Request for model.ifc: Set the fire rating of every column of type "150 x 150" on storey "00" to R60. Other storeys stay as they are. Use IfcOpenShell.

First a look at what the model holds.

```python
import ifcopenshell
import ifcopenshell.util.element

model = ifcopenshell.open("model.ifc")
print(model.schema)
storey = next(s for s in model.by_type("IfcBuildingStorey") if s.Name == "00")
columns = [e for e in ifcopenshell.util.element.get_decomposition(storey) if e.is_a("IfcColumn")]
seen = {}
for e in columns:
    element_type = ifcopenshell.util.element.get_type(e)
    key = (element_type.Name if element_type != e and element_type else None, ifcopenshell.util.element.get_pset(e, "Pset_ColumnCommon", "FireRating"))
    seen[key] = seen.get(key, 0) + 1
for (name, value), count in sorted(seen.items(), key=str):
    print(count, "x", name, "|", value)
```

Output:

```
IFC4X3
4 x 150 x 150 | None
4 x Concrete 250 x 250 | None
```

```python
import ifcopenshell
import ifcopenshell.api.pset
import ifcopenshell.util.element

model = ifcopenshell.open("model.ifc")

storey = next(s for s in model.by_type("IfcBuildingStorey") if s.Name == "00")
columns = [e for e in ifcopenshell.util.element.get_decomposition(storey) if e.is_a("IfcColumn")]

count = 0
for e in columns:
    element_type = ifcopenshell.util.element.get_type(e)
    if element_type in (None, e) or element_type.Name != "150 x 150":
        continue
    # add_pset returns the element's existing set when there is one.
    pset = ifcopenshell.api.pset.add_pset(model, product=e, name="Pset_ColumnCommon")
    ifcopenshell.api.pset.edit_pset(model, pset=pset, properties={"FireRating": "R60"})
    count += 1

print(count, "columns updated")

model.write("model-out.ifc")
```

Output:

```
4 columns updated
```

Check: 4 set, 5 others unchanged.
